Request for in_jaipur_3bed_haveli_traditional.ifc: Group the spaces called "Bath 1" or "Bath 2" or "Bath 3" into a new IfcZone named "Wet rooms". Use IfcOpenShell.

First a look at what the model holds.

```python
import ifcopenshell

model = ifcopenshell.open("in_jaipur_3bed_haveli_traditional.ifc")
print(model.schema)
seen = {}
for space in model.by_type("IfcSpace"):
    seen[space.LongName] = seen.get(space.LongName, 0) + 1
for name, count in sorted(seen.items(), key=str):
    print(count, "x", name)
print("zones:", [z.Name for z in model.by_type("IfcZone")][:20])
```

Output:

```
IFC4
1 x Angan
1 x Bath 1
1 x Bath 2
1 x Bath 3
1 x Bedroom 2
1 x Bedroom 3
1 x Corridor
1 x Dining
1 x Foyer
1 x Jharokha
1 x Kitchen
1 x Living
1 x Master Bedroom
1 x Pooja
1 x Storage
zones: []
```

```python
import ifcopenshell
import ifcopenshell.api.group
import ifcopenshell.api.root

model = ifcopenshell.open("in_jaipur_3bed_haveli_traditional.ifc")

names = {"Bath 1", "Bath 2", "Bath 3"}
spaces = [s for s in model.by_type("IfcSpace") if s.LongName in names]

zone = ifcopenshell.api.root.create_entity(model, ifc_class="IfcZone", name="Wet rooms")
ifcopenshell.api.group.assign_group(model, products=spaces, group=zone)
print(len(spaces), "spaces in", zone.Name)

model.write("in_jaipur_3bed_haveli_traditional_v2.ifc")
```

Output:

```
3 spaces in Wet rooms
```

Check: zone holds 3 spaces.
